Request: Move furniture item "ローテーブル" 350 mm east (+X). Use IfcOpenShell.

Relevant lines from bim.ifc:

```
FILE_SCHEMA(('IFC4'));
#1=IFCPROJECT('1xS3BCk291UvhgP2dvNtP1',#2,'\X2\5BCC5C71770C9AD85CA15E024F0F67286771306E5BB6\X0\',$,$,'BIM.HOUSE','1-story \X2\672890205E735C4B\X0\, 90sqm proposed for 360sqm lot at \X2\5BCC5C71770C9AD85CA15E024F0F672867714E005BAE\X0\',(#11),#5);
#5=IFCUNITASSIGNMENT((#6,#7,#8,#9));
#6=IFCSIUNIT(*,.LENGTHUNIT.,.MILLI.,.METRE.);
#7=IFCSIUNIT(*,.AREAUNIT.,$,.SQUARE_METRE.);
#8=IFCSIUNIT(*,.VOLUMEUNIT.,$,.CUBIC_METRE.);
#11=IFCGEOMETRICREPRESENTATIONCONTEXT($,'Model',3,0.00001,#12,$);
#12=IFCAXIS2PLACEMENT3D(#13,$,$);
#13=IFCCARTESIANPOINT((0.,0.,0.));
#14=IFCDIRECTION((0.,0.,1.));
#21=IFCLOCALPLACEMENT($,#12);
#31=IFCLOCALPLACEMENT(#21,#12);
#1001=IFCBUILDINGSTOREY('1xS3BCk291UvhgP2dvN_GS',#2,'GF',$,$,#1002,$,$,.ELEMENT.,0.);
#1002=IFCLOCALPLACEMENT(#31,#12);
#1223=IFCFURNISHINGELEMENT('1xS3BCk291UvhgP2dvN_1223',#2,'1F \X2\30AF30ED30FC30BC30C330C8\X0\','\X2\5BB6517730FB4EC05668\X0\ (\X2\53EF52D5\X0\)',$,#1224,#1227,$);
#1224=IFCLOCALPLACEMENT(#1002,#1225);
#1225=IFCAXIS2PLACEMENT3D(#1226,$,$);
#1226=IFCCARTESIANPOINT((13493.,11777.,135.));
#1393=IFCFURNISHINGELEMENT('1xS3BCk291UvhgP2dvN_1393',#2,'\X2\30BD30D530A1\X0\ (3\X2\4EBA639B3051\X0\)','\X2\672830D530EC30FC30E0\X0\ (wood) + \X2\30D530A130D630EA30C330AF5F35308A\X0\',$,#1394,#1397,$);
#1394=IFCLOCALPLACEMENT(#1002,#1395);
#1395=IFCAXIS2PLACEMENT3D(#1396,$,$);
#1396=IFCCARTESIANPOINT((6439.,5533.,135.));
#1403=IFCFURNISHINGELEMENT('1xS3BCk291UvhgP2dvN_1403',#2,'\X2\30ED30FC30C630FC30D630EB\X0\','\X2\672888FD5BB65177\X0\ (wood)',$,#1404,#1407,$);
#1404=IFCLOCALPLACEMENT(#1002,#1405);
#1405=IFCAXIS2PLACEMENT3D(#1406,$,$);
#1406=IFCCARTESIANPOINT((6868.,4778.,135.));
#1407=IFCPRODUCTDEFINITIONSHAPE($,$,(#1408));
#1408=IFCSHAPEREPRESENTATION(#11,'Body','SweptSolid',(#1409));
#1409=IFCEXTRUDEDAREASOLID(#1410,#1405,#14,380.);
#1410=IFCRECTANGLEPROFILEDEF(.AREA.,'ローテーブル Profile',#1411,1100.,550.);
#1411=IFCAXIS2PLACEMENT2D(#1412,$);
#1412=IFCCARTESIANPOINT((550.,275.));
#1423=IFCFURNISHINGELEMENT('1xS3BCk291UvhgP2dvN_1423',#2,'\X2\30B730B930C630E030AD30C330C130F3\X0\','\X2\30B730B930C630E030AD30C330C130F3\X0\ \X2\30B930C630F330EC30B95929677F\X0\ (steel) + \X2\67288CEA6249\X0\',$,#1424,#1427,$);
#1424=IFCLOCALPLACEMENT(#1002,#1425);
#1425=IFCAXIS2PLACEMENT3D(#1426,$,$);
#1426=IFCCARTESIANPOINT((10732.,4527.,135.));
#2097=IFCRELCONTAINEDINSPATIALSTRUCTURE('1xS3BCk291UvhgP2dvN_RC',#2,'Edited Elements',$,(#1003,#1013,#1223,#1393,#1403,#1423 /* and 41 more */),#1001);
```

```python
import ifcopenshell
import ifcopenshell.api.geometry
import ifcopenshell.util.placement

model = ifcopenshell.open("bim.ifc")

item = model.by_guid("1xS3BCk291UvhgP2dvN_1403")
matrix = ifcopenshell.util.placement.get_local_placement(item.ObjectPlacement)
matrix[0, 3] += 350.0
ifcopenshell.api.geometry.edit_object_placement(model, product=item, matrix=matrix, is_si=False)

print(ifcopenshell.util.placement.get_local_placement(item.ObjectPlacement).round(3) + 0.0)

model.write("bim_edited.ifc")
```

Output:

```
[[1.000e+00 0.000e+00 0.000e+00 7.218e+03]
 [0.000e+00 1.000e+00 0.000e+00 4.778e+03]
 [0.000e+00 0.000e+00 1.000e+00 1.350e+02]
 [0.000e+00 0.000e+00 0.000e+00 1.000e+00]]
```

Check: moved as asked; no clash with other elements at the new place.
